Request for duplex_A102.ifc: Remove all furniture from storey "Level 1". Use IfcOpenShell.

First a look at what the model holds.

```python
import ifcopenshell
import ifcopenshell.util.element

model = ifcopenshell.open("duplex_A102.ifc")
print(model.schema)
storey = next(s for s in model.by_type("IfcBuildingStorey") if s.Name == "Level 1")
furniture = [e for e in ifcopenshell.util.element.get_decomposition(storey) if e.is_a("IfcFurnishingElement")]
seen = {}
for e in furniture:
    element_type = ifcopenshell.util.element.get_type(e)
    name = element_type.Name if element_type not in (None, e) else None
    seen[name] = seen.get(name, 0) + 1
for name, count in sorted(seen.items(), key=str):
    print(count, "x", name)
```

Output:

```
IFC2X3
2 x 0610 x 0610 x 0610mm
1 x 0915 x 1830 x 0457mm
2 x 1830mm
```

```python
import ifcopenshell
import ifcopenshell.api.root
import ifcopenshell.util.element

model = ifcopenshell.open("duplex_A102.ifc")

storey = next(s for s in model.by_type("IfcBuildingStorey") if s.Name == "Level 1")
furniture = [e for e in ifcopenshell.util.element.get_decomposition(storey) if e.is_a("IfcFurnishingElement")]

for e in furniture:
    ifcopenshell.api.root.remove_product(model, product=e)
print(len(furniture), "removed")

model.write("duplex_A102-out.ifc")
```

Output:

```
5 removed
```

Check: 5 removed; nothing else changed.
